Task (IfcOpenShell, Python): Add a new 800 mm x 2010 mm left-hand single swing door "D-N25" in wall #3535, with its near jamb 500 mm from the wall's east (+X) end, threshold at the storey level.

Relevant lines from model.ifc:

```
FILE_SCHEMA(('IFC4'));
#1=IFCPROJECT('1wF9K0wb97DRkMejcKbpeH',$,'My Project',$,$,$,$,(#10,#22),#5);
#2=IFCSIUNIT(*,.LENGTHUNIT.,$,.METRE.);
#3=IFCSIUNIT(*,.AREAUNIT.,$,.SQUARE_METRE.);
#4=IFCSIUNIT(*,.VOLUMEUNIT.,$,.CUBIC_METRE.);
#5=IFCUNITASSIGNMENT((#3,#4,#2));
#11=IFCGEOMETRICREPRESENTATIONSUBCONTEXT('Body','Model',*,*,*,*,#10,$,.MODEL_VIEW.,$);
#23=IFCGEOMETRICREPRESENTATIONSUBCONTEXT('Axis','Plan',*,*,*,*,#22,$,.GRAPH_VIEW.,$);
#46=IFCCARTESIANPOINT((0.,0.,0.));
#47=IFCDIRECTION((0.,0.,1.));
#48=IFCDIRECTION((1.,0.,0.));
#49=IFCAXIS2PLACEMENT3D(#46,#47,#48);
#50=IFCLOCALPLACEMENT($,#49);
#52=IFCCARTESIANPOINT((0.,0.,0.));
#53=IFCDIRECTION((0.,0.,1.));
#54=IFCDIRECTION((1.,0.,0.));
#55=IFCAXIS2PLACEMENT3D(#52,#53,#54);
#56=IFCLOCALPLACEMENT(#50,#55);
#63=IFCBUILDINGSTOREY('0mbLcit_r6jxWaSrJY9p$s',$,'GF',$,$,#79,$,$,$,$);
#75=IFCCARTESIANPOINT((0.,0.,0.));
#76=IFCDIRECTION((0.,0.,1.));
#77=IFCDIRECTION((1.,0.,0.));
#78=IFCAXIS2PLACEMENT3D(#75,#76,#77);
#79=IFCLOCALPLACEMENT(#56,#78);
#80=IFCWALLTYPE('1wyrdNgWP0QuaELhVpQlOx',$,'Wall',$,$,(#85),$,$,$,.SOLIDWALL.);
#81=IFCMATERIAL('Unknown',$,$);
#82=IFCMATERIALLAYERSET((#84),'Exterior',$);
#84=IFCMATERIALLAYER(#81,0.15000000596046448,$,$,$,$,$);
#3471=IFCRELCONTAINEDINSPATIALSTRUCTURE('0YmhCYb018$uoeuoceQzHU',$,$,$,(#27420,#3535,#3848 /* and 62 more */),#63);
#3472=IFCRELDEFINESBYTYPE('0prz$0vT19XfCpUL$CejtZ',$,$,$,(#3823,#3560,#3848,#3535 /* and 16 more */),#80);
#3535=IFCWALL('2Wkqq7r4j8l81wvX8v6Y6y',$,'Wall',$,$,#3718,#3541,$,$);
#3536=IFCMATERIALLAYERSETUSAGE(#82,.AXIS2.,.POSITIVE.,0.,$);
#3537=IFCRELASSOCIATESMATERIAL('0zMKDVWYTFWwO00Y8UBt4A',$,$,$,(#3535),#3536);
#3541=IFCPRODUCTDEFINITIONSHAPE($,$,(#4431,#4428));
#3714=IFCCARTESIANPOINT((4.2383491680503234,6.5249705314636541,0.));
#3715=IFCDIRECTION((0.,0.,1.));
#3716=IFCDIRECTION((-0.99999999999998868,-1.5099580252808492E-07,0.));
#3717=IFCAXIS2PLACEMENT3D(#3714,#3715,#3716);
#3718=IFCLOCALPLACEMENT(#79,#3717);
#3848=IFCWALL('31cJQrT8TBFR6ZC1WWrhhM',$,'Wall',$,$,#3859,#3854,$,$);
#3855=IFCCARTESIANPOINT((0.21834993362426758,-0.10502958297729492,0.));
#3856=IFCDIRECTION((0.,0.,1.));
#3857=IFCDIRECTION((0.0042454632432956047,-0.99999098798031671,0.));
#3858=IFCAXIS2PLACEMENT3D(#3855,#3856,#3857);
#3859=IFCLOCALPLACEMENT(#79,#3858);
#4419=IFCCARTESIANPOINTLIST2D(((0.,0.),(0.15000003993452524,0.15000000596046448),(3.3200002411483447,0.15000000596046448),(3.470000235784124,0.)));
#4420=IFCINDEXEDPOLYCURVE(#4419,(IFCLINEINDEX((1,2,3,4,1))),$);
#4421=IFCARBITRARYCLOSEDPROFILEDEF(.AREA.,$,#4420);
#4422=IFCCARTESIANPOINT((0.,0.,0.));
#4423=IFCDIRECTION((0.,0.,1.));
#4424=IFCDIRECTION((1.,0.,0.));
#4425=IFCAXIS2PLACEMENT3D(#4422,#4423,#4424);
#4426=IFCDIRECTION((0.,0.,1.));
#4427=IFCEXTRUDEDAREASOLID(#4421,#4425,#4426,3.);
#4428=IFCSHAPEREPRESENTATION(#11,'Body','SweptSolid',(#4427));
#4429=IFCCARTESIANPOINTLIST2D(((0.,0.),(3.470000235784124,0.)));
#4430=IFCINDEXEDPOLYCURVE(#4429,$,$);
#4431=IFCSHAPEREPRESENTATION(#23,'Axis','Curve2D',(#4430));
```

```python
import numpy as np
import ifcopenshell
import ifcopenshell.api.feature
import ifcopenshell.api.geometry
import ifcopenshell.api.root
import ifcopenshell.api.spatial
import ifcopenshell.geom
import ifcopenshell.util.element
import ifcopenshell.util.placement
import ifcopenshell.util.representation
import ifcopenshell.util.shape
import ifcopenshell.util.unit

model = ifcopenshell.open("model.ifc")
unit_scale = ifcopenshell.util.unit.calculate_unit_scale(model)
settings = ifcopenshell.geom.settings()


def volume(element):
    """Net volume in cubic metres, openings subtracted."""
    shape = ifcopenshell.geom.create_shape(settings, element)
    return ifcopenshell.util.shape.get_volume(shape.geometry)


wall = model.by_guid("2Wkqq7r4j8l81wvX8v6Y6y")
storey = ifcopenshell.util.element.get_container(wall, ifc_class="IfcBuildingStorey")
context = ifcopenshell.util.representation.get_context(model, "Model", "Body", "MODEL_VIEW")
before = volume(wall)

width, height, from_end, sill = 0.8, 2.01, 0.5, 0.0  # metres

# The wall runs along its own X axis, and the end named is its -X end.
wall_shape = ifcopenshell.geom.create_shape(settings, wall)
x, y, z = ifcopenshell.util.shape.get_vertices(wall_shape.geometry).T
start = x.min() + from_end
face, thickness = float(y.min()), float(y.max() - y.min())
wall_matrix = ifcopenshell.util.placement.get_local_placement(wall.ObjectPlacement)
level = ifcopenshell.util.placement.get_local_placement(storey.ObjectPlacement)[2, 3]


def in_wall(x, y):
    """Placement at x, y metres in the wall's axes, at sill height."""
    matrix = wall_matrix.copy()
    matrix[:, 3] = wall_matrix @ np.array([x / unit_scale, y / unit_scale, 0.0, 1.0])
    matrix[2, 3] = level + sill / unit_scale
    return matrix


# Opening: a box that overshoots both wall faces by 50 mm.
opening = ifcopenshell.api.root.create_entity(model, ifc_class="IfcOpeningElement", predefined_type="OPENING")
box = ifcopenshell.api.geometry.add_wall_representation(
    model, context=context, length=width, height=height, thickness=thickness + 0.1
)
ifcopenshell.api.geometry.assign_representation(model, product=opening, representation=box)
ifcopenshell.api.geometry.edit_object_placement(model, product=opening, matrix=in_wall(start, face - 0.05), is_si=False)
ifcopenshell.api.feature.add_feature(model, feature=opening, element=wall)

door = ifcopenshell.api.root.create_entity(model, ifc_class="IfcDoor", name="D-N25", predefined_type="DOOR")
door.OverallWidth, door.OverallHeight = width / unit_scale, height / unit_scale
door.OperationType = "SINGLE_SWING_LEFT"
body = ifcopenshell.api.geometry.add_door_representation(
    model,
    context=context,
    overall_width=door.OverallWidth,
    overall_height=door.OverallHeight,
    operation_type="SINGLE_SWING_LEFT",
    lining_properties={"LiningDepth": thickness / unit_scale, "ThresholdDepth": thickness / unit_scale},
)
ifcopenshell.api.geometry.assign_representation(model, product=door, representation=body)
ifcopenshell.api.spatial.assign_container(model, products=[door], relating_structure=storey)
ifcopenshell.api.feature.add_filling(model, opening=opening, element=door)

# The lining spans the wall, so the door starts at the wall face.
ifcopenshell.api.geometry.edit_object_placement(model, product=door, matrix=in_wall(start, face), is_si=False)

after = volume(wall)

print(f"wall volume {before:.3f} -> {after:.3f} m3")

model.write("model_rev.ifc")
```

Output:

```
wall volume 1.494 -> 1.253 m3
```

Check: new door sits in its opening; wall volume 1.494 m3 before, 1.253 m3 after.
